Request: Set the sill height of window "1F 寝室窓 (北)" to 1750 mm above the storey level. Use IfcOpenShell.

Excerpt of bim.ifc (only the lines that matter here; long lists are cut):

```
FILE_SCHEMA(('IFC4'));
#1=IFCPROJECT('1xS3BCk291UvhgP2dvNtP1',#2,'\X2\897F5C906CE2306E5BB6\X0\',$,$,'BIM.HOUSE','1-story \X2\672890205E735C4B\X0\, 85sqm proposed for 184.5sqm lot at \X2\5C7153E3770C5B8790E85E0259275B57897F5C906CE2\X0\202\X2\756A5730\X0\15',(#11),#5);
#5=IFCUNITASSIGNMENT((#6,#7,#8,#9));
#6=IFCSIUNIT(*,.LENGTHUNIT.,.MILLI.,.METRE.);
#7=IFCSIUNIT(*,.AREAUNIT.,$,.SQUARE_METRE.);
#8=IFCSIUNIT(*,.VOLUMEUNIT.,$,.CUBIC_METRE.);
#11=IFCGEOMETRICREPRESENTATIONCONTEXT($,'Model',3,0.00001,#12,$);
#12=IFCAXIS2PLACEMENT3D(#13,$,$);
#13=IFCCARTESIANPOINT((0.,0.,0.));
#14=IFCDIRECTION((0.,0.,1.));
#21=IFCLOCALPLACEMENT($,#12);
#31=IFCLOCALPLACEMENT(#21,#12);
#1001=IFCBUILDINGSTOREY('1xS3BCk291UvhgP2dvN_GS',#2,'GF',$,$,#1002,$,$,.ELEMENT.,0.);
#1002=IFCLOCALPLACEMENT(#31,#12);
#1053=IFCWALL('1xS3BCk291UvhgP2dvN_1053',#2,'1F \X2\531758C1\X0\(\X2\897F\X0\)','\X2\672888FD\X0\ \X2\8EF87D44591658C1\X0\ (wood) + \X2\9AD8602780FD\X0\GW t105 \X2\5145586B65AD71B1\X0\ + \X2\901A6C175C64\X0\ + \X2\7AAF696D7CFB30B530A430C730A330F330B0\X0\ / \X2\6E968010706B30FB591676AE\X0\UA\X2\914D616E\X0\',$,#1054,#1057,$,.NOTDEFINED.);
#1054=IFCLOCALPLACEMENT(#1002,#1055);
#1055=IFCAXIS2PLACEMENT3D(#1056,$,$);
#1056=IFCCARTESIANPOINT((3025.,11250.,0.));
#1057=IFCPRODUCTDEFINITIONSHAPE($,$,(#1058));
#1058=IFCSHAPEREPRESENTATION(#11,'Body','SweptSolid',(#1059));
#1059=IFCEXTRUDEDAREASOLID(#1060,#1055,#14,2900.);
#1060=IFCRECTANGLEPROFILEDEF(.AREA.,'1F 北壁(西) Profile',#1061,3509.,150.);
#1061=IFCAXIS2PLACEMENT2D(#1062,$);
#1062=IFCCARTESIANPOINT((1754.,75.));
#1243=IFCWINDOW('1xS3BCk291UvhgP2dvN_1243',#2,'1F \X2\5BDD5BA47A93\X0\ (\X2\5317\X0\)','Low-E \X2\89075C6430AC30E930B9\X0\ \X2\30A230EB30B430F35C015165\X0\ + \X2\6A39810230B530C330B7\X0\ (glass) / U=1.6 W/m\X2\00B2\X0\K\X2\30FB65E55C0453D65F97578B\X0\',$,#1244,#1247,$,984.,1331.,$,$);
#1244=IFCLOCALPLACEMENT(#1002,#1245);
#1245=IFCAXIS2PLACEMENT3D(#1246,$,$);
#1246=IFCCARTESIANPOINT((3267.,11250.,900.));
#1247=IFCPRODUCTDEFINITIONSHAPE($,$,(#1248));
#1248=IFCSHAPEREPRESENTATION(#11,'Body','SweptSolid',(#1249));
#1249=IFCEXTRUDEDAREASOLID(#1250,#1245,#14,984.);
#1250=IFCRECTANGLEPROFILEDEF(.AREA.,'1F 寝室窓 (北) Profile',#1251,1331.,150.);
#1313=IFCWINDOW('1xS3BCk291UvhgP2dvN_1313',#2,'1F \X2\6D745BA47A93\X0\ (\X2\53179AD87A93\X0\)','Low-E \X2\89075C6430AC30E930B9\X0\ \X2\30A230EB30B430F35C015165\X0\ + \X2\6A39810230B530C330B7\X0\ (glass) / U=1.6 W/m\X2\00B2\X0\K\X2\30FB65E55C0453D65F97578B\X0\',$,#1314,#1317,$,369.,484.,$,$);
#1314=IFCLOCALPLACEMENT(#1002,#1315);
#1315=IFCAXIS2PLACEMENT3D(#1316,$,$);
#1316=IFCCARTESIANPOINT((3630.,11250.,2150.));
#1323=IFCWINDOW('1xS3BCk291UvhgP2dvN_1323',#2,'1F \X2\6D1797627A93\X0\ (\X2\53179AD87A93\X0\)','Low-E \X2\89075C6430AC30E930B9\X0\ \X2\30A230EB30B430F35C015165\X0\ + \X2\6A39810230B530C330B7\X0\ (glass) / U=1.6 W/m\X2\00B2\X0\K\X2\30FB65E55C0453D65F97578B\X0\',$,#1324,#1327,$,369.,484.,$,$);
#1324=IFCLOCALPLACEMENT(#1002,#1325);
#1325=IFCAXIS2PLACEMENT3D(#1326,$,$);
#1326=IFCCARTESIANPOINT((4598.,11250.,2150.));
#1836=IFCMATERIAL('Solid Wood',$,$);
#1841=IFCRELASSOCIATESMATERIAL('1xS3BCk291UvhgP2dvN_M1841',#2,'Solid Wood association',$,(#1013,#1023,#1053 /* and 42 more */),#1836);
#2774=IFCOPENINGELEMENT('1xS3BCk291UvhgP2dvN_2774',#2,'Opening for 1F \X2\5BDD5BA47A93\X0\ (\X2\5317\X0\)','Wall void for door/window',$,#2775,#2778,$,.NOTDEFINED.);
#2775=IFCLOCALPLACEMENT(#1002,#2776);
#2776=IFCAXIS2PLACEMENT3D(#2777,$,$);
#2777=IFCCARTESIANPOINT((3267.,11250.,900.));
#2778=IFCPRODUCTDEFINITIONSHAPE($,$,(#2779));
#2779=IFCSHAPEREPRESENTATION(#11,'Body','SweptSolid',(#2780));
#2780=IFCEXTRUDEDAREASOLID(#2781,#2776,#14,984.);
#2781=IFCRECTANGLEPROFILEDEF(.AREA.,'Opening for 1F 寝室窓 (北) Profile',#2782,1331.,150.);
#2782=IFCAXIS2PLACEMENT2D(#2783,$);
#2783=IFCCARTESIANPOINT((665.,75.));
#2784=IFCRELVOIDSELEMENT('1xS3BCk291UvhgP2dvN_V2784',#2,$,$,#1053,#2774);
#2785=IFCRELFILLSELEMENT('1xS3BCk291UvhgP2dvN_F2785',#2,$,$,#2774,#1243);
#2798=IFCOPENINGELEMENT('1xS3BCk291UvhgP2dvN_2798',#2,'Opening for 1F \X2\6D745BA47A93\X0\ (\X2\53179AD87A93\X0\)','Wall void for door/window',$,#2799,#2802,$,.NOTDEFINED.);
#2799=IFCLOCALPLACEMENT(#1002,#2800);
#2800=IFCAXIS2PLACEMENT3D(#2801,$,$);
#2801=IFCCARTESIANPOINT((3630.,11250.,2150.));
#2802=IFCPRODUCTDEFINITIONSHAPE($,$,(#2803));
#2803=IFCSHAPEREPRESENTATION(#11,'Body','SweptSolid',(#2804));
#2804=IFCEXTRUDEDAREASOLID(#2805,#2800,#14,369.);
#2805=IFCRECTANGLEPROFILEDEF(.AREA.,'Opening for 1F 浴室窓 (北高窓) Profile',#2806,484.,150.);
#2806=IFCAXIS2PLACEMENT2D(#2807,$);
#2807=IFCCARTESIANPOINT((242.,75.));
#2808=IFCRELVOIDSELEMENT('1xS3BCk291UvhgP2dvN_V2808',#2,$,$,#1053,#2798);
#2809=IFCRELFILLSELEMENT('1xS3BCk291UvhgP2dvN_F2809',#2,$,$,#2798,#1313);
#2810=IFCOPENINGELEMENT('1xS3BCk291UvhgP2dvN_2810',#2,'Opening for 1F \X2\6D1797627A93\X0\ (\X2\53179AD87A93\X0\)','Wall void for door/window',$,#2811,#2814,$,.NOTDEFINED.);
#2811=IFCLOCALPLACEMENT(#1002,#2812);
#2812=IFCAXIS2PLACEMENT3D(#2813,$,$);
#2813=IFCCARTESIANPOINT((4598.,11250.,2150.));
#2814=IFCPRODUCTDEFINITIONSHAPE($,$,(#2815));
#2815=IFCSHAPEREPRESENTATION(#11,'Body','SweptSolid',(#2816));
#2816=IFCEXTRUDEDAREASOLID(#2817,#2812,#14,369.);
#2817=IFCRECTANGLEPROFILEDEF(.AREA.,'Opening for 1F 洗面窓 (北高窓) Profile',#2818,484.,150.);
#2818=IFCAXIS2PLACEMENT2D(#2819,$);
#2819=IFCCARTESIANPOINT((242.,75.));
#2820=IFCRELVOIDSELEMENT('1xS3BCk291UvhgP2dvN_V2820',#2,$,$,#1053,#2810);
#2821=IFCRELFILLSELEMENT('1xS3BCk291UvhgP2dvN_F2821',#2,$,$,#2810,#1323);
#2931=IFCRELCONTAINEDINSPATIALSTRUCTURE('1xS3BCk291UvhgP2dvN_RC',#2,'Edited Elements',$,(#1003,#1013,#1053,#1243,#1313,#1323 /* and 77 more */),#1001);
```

```python
import numpy as np
import ifcopenshell
import ifcopenshell.api.geometry
import ifcopenshell.geom
import ifcopenshell.util.element
import ifcopenshell.util.placement
import ifcopenshell.util.shape
import ifcopenshell.util.unit

model = ifcopenshell.open("bim.ifc")
unit_scale = ifcopenshell.util.unit.calculate_unit_scale(model)

window = model.by_guid("1xS3BCk291UvhgP2dvN_1243")
opening = window.FillsVoids[0].RelatingOpeningElement
storey = ifcopenshell.util.element.get_container(window, ifc_class="IfcBuildingStorey")
level = ifcopenshell.util.placement.get_local_placement(storey.ObjectPlacement)[2, 3]

# The opening's origin need not be at the sill, so measure its lowest point.
shape = ifcopenshell.geom.create_shape(ifcopenshell.geom.settings(), opening)
bottom = ifcopenshell.util.shape.get_shape_bottom_elevation(shape, shape.geometry) / unit_scale
dz = level + 1.75 / unit_scale - bottom

shift = np.array([0.0, 0.0, dz])
# The window is not placed relative to its opening, so move both.
for product in (opening, window):
    matrix = ifcopenshell.util.placement.get_local_placement(product.ObjectPlacement)
    matrix[:3, 3] += shift
    ifcopenshell.api.geometry.edit_object_placement(model, product=product, matrix=matrix, is_si=False)

print(f"moved by {dz * unit_scale:+.3f} m")

model.write("bim_v2.ifc")
```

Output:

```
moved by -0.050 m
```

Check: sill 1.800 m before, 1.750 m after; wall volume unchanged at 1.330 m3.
